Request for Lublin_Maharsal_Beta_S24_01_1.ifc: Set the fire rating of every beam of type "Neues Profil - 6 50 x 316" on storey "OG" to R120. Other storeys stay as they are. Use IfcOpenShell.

First a look at what the model holds.

```python
import ifcopenshell
import ifcopenshell.util.element

model = ifcopenshell.open("Lublin_Maharsal_Beta_S24_01_1.ifc")
print(model.schema)
storey = next(s for s in model.by_type("IfcBuildingStorey") if s.Name == "OG")
beams = [e for e in ifcopenshell.util.element.get_decomposition(storey) if e.is_a("IfcBeam")]
seen = {}
for e in beams:
    element_type = ifcopenshell.util.element.get_type(e)
    key = (element_type.Name if element_type != e and element_type else None, ifcopenshell.util.element.get_pset(e, "Pset_BeamCommon", "FireRating"))
    seen[key] = seen.get(key, 0) + 1
for (name, value), count in sorted(seen.items(), key=str):
    print(count, "x", name, "|", value)
```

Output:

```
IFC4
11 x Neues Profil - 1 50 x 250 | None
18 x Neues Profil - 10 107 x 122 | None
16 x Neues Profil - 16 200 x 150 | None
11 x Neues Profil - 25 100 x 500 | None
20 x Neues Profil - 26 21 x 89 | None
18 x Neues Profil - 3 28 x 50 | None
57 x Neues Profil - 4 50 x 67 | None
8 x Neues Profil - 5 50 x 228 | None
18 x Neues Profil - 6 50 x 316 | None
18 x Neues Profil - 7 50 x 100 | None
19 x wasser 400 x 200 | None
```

```python
import ifcopenshell
import ifcopenshell.api.pset
import ifcopenshell.util.element

model = ifcopenshell.open("Lublin_Maharsal_Beta_S24_01_1.ifc")

storey = next(s for s in model.by_type("IfcBuildingStorey") if s.Name == "OG")
beams = [e for e in ifcopenshell.util.element.get_decomposition(storey) if e.is_a("IfcBeam")]

count = 0
for e in beams:
    element_type = ifcopenshell.util.element.get_type(e)
    if element_type in (None, e) or element_type.Name != "Neues Profil - 6 50 x 316":
        continue
    # add_pset returns the element's existing set when there is one.
    pset = ifcopenshell.api.pset.add_pset(model, product=e, name="Pset_BeamCommon")
    ifcopenshell.api.pset.edit_pset(model, pset=pset, properties={"FireRating": "R120"})
    count += 1

print(count, "beams updated")

model.write("Lublin_Maharsal_Beta_S24_01_1_updated.ifc")
```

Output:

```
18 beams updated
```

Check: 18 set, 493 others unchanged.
